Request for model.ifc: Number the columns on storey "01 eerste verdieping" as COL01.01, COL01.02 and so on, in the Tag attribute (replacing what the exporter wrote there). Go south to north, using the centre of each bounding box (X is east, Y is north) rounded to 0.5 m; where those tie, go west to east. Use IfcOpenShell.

First a look at what the model holds.

```python
import ifcopenshell
import ifcopenshell.util.element
import ifcopenshell.util.placement

model = ifcopenshell.open("model.ifc")
print(model.schema)
storey = next(s for s in model.by_type("IfcBuildingStorey") if s.Name == "01 eerste verdieping")
columns = [e for e in ifcopenshell.util.element.get_decomposition(storey) if e.is_a("IfcColumn")]
for e in sorted(columns, key=lambda e: e.id()):
    origin = ifcopenshell.util.placement.get_local_placement(e.ObjectPlacement)[:3, 3]
    print(e.id(), e.Tag, e.Name, origin.round(2) + 0.0, sep=" | ")
```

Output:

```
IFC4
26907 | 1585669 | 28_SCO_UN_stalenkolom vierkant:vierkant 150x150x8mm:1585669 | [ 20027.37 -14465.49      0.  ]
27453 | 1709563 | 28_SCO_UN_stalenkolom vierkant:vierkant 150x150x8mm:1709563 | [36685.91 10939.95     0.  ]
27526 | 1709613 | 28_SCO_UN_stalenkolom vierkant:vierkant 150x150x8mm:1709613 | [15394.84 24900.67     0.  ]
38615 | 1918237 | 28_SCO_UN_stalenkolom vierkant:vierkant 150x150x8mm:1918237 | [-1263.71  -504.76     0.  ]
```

```python
import ifcopenshell
import ifcopenshell.geom
import ifcopenshell.util.element
import ifcopenshell.util.shape

model = ifcopenshell.open("model.ifc")
settings = ifcopenshell.geom.settings()
settings.set("use-world-coords", True)


def centre(element):
    shape = ifcopenshell.geom.create_shape(settings, element)
    return ifcopenshell.util.shape.get_bbox_centroid(shape.geometry)


storey = next(s for s in model.by_type("IfcBuildingStorey") if s.Name == "01 eerste verdieping")
columns = [e for e in ifcopenshell.util.element.get_decomposition(storey) if e.is_a("IfcColumn")]

# Insertion points can sit at a corner or the storey origin, so sort by the geometry (in metres).
centres = {e: centre(e) for e in columns}
columns.sort(key=lambda e: (round(centres[e][1] / 0.5), centres[e][0]))

for i, e in enumerate(columns, start=1):
    number = f"COL01.{i:02d}"
    e.Tag = number
    print(e.id(), number)

model.write("model_edited.ifc")
```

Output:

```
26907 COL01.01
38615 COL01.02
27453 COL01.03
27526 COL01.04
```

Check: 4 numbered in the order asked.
